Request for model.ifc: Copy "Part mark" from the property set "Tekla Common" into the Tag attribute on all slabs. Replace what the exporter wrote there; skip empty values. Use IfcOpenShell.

First a look at what the model holds.

```python
import ifcopenshell
import ifcopenshell.util.element

model = ifcopenshell.open("model.ifc")
print(model.schema)
slabs = model.by_type("IfcSlab")
print(len(slabs), "slabs")
for e in slabs[:8]:
    source = ifcopenshell.util.element.get_pset(e, "Tekla Common", "Part mark")
    target = e.Tag
    print(e.id(), repr(source), repr(target), sep=" | ")
```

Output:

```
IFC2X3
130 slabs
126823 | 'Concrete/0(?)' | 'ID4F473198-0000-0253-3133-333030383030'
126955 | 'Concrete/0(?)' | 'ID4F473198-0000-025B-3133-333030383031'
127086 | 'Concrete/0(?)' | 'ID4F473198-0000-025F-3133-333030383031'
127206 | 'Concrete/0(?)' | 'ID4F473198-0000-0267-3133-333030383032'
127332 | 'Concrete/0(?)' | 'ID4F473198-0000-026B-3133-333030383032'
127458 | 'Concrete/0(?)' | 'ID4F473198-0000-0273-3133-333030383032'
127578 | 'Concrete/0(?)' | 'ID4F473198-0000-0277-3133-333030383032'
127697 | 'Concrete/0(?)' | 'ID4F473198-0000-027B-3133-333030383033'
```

```python
import ifcopenshell
import ifcopenshell.util.element

model = ifcopenshell.open("model.ifc")

count = 0
for e in model.by_type("IfcSlab"):
    value = ifcopenshell.util.element.get_pset(e, "Tekla Common", "Part mark")
    current = e.Tag
    if not value or not value.strip() or current == value:
        continue
    e.Tag = value
    count += 1

print(count, "slabs updated")

model.write("model-out.ifc")
```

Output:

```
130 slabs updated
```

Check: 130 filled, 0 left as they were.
